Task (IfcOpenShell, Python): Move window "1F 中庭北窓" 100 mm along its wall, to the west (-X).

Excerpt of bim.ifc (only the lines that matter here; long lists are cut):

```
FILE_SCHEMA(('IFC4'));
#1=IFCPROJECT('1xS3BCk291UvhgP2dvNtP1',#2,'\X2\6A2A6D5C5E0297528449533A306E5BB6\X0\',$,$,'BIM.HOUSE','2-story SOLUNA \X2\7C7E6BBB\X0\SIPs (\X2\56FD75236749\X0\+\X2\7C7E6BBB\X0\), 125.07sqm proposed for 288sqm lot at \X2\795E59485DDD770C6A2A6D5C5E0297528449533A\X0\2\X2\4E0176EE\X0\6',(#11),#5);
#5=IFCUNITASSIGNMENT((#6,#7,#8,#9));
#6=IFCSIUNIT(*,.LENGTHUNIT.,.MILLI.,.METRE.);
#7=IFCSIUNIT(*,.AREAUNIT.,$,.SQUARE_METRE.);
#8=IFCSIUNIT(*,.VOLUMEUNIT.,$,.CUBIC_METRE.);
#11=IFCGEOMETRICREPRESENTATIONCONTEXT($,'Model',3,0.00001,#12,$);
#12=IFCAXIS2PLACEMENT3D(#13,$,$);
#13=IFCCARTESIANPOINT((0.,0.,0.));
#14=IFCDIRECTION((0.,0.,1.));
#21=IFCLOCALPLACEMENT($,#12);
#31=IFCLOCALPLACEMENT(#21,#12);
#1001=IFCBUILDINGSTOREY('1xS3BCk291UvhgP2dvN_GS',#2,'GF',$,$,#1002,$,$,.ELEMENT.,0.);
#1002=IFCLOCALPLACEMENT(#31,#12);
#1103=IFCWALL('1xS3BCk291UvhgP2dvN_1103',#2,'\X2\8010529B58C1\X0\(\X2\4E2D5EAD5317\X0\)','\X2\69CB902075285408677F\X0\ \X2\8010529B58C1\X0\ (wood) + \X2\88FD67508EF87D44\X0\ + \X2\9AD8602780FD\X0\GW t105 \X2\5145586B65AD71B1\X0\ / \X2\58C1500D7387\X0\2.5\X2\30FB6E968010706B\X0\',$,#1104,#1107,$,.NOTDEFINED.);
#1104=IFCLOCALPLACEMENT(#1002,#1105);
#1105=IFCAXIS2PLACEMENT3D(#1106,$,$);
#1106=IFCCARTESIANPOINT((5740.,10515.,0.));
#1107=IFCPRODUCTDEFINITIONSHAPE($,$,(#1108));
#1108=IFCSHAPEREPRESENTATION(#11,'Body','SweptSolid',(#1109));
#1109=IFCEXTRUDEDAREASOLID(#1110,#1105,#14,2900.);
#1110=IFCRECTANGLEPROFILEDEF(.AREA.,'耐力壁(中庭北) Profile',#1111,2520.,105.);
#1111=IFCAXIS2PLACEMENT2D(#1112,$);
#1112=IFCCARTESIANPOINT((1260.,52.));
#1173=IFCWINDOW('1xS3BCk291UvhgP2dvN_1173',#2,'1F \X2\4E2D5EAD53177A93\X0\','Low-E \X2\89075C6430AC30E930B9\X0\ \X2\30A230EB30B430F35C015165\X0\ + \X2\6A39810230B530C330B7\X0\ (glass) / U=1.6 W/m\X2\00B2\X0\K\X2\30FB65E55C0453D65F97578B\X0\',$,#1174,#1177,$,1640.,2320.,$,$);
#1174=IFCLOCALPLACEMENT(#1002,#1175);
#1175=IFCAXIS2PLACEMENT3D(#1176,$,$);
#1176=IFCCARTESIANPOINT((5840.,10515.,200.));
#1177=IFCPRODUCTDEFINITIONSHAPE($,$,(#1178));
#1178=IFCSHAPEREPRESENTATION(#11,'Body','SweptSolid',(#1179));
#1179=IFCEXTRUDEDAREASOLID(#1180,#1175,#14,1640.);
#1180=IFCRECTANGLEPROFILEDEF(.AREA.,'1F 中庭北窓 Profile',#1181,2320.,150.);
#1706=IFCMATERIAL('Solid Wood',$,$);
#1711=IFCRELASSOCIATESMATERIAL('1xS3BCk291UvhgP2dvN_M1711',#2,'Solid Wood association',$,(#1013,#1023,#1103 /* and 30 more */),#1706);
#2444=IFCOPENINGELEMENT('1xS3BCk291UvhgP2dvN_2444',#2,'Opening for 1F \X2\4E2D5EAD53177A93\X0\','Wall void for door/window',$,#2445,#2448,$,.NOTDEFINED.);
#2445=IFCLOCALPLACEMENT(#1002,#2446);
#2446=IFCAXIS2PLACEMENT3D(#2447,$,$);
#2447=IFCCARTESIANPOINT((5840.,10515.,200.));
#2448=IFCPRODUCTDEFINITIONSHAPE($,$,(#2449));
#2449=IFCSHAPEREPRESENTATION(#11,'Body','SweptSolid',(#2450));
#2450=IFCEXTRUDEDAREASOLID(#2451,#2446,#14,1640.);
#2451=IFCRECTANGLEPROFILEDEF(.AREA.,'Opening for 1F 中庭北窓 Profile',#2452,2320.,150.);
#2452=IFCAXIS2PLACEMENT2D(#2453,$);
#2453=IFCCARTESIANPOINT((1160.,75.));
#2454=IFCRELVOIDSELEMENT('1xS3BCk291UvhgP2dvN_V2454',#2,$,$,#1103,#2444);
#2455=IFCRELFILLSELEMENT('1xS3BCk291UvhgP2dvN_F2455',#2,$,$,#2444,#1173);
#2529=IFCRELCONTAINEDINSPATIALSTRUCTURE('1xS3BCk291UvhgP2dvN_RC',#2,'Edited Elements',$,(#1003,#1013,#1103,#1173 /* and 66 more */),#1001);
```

```python
import ifcopenshell
import ifcopenshell.api.geometry
import ifcopenshell.util.placement

model = ifcopenshell.open("bim.ifc")

window = model.by_id(1173)
opening = window.FillsVoids[0].RelatingOpeningElement
wall = opening.VoidsElements[0].RelatingBuildingElement

wall_matrix = ifcopenshell.util.placement.get_local_placement(wall.ObjectPlacement)
shift = wall_matrix[:3, 0] * -100.0
before = ifcopenshell.util.placement.get_local_placement(window.ObjectPlacement)[:3, 3].copy()

# The window is not placed relative to its opening, so move both.
for product in (opening, window):
    matrix = ifcopenshell.util.placement.get_local_placement(product.ObjectPlacement)
    matrix[:3, 3] += shift
    ifcopenshell.api.geometry.edit_object_placement(model, product=product, matrix=matrix, is_si=False)

after = ifcopenshell.util.placement.get_local_placement(window.ObjectPlacement)[:3, 3]
print("window moved by", (after - before).round(3) + 0.0)

model.write("bim-out.ifc")
```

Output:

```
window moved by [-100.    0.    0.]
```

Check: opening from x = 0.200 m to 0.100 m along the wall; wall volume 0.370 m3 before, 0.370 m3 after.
